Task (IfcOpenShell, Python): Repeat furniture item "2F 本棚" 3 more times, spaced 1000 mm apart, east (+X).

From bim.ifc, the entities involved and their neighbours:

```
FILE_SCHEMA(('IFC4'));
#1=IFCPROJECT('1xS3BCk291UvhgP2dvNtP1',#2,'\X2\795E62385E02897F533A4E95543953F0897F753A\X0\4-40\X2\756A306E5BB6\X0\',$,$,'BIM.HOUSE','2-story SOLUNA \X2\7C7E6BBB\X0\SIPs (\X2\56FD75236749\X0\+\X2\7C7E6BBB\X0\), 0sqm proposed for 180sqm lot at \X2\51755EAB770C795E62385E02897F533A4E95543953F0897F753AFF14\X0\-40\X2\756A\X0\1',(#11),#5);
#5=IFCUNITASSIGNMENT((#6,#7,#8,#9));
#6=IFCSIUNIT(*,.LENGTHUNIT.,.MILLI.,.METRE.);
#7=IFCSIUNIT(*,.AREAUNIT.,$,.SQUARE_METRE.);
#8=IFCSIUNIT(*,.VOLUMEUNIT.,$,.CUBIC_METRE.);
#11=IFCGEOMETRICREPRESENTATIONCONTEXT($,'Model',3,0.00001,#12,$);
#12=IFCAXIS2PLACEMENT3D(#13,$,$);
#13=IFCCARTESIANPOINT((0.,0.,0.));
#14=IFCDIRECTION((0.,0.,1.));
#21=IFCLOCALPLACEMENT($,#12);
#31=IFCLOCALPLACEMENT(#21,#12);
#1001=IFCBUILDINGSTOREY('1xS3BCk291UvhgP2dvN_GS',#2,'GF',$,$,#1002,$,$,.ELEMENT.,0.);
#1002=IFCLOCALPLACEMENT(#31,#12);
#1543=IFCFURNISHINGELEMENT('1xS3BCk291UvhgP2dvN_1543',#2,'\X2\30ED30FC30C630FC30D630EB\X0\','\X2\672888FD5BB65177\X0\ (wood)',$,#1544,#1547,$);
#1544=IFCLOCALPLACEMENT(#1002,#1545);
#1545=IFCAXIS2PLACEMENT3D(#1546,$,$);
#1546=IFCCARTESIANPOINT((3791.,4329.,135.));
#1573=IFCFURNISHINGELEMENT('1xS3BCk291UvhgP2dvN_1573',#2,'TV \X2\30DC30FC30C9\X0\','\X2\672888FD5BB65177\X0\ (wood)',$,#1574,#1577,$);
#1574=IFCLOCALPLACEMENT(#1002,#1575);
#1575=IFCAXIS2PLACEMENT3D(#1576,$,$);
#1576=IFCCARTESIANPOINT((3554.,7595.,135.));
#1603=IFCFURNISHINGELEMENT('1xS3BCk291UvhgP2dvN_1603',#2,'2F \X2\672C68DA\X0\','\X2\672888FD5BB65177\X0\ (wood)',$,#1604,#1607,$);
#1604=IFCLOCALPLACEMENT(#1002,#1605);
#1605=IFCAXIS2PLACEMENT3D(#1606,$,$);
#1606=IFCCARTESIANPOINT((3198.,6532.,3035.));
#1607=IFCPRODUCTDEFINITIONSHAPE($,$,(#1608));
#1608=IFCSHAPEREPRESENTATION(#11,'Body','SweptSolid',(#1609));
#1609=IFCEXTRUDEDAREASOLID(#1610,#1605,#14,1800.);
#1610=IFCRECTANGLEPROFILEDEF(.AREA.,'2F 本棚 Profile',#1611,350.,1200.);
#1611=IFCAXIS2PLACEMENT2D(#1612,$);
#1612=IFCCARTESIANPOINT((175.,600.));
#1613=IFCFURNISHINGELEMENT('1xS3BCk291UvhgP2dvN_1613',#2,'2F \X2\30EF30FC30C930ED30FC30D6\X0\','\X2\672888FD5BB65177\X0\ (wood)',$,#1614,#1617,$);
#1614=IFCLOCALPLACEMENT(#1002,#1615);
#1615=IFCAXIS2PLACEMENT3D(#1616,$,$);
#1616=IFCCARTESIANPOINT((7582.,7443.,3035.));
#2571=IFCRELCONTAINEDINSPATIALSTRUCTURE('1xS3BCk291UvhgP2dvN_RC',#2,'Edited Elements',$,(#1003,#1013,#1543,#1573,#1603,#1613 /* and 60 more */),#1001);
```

```python
import numpy as np
import ifcopenshell
import ifcopenshell.api.geometry
import ifcopenshell.api.root
import ifcopenshell.util.element
import ifcopenshell.util.placement
import ifcopenshell.util.unit

model = ifcopenshell.open("bim.ifc")
unit_scale = ifcopenshell.util.unit.calculate_unit_scale(model)


def reuse_history(source, copy):
    """copy_class also copies each property set's owner history, people and application; keep the originals."""
    for rel in copy.IsDefinedBy:
        if rel.is_a("IfcRelDefinesByProperties") and (history := rel.RelatingPropertyDefinition.OwnerHistory):
            rel.RelatingPropertyDefinition.OwnerHistory = source.OwnerHistory
            ifcopenshell.util.element.remove_deep2(model, history)


source = model.by_guid("1xS3BCk291UvhgP2dvN_1603")
base = ifcopenshell.util.placement.get_local_placement(source.ObjectPlacement)
step = np.array([1.0, 0.0, 0.0]) * 1 / unit_scale

for i in range(1, 4):
    copy = ifcopenshell.api.root.copy_class(model, product=source)
    copy.Representation = ifcopenshell.util.element.copy_deep(
        model, source.Representation, exclude=["IfcGeometricRepresentationContext", "IfcRepresentationMap"]
    )
    reuse_history(source, copy)
    matrix = base.copy()
    matrix[:3, 3] += i * step
    print("added at", matrix[:3, 3].round(3) + 0.0)
    ifcopenshell.api.geometry.edit_object_placement(model, product=copy, matrix=matrix, is_si=False)

model.write("bim_updated.ifc")
```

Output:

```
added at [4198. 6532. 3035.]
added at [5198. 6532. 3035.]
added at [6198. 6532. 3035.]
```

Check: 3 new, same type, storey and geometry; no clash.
